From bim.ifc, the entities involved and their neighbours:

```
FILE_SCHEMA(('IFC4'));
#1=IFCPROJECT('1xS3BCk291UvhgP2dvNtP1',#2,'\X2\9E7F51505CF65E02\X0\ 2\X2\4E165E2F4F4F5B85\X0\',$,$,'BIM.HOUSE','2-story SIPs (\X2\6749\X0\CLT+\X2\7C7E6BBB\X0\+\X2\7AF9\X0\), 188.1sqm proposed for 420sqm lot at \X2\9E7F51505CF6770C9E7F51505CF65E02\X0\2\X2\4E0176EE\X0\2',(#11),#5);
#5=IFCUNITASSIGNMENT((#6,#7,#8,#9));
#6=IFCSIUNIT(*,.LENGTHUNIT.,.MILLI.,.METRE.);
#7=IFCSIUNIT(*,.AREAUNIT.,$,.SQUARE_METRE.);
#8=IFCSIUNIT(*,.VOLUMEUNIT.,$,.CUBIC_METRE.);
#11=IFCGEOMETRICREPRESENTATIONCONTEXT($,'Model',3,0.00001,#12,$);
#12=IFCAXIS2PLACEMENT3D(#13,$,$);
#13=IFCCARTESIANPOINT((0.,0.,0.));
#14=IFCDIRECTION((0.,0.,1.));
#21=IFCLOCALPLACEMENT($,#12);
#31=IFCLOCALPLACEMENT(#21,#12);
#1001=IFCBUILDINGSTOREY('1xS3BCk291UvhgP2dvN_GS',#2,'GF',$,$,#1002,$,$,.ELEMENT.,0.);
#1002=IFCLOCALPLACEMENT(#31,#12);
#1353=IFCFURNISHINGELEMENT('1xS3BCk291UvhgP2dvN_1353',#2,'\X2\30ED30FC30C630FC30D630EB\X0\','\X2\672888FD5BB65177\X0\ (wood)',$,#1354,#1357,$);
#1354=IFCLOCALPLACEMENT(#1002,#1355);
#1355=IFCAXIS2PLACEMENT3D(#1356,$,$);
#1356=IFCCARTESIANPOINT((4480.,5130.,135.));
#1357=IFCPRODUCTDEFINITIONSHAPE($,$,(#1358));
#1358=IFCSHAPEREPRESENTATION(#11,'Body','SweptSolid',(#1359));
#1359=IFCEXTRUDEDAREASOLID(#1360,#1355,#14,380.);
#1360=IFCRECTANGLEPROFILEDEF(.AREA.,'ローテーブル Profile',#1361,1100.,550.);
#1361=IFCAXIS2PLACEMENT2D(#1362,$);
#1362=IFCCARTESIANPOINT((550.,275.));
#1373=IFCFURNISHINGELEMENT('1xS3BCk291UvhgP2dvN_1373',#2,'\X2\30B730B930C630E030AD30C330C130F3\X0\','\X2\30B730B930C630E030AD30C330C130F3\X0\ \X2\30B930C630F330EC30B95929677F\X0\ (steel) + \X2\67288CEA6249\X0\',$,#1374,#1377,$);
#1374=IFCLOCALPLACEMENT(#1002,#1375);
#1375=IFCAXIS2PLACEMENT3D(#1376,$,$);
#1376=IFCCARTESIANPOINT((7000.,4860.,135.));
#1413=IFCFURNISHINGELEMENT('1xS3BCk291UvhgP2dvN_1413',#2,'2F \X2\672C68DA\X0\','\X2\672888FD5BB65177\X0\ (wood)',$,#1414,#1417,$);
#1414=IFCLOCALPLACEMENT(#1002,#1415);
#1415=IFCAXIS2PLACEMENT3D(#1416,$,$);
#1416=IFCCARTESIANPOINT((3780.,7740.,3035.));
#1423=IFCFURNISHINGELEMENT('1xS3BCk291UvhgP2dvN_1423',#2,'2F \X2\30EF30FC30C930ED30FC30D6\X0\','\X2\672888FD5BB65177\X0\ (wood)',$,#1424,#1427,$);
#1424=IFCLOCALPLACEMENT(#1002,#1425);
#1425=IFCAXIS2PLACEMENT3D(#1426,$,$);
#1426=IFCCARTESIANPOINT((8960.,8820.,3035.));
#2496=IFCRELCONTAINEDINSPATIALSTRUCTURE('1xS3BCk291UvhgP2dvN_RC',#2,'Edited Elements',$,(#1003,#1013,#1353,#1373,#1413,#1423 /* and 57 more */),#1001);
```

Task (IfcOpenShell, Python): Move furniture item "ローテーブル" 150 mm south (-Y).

```python
import ifcopenshell
import ifcopenshell.api.geometry
import ifcopenshell.util.placement
import ifcopenshell.util.unit

model = ifcopenshell.open("bim.ifc")
unit_scale = ifcopenshell.util.unit.calculate_unit_scale(model)

item = model.by_guid("1xS3BCk291UvhgP2dvN_1353")
matrix = ifcopenshell.util.placement.get_local_placement(item.ObjectPlacement)
matrix[1, 3] -= 0.15 / unit_scale
ifcopenshell.api.geometry.edit_object_placement(model, product=item, matrix=matrix, is_si=False)

print(ifcopenshell.util.placement.get_local_placement(item.ObjectPlacement).round(3) + 0.0)

model.write("bim_updated.ifc")
```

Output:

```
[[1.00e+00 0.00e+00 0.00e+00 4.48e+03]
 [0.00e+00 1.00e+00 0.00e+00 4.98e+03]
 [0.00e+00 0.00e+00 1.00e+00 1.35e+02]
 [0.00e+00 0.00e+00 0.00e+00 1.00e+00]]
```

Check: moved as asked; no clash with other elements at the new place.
